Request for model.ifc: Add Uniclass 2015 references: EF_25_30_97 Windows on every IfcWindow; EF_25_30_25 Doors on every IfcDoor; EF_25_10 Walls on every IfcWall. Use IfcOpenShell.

First a look at what the model holds.

```python
import ifcopenshell

model = ifcopenshell.open("model.ifc")
print(model.schema)
print("classifications:", [c.Name for c in model.by_type("IfcClassification")])
for ifc_class in ("IfcDoor", "IfcRoof", "IfcStair", "IfcWall", "IfcWindow"):
    print(ifc_class, len(model.by_type(ifc_class)))
```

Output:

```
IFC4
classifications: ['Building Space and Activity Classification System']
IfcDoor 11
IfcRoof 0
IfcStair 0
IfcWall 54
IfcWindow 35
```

```python
import ifcopenshell
import ifcopenshell.api.classification

model = ifcopenshell.open("model.ifc")

system = ifcopenshell.api.classification.add_classification(model, classification="Uniclass 2015")

codes = {
    "IfcWindow": ("EF_25_30_97", "Windows"),
    "IfcDoor": ("EF_25_30_25", "Doors"),
    "IfcWall": ("EF_25_10", "Walls"),
}
for ifc_class, (code, name) in codes.items():
    products = model.by_type(ifc_class)
    ifcopenshell.api.classification.add_reference(
        model, products=products, classification=system, identification=code, name=name
    )
    print(code, len(products))

model.write("model_edited.ifc")
```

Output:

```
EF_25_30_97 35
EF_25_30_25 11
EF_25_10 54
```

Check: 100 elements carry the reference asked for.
